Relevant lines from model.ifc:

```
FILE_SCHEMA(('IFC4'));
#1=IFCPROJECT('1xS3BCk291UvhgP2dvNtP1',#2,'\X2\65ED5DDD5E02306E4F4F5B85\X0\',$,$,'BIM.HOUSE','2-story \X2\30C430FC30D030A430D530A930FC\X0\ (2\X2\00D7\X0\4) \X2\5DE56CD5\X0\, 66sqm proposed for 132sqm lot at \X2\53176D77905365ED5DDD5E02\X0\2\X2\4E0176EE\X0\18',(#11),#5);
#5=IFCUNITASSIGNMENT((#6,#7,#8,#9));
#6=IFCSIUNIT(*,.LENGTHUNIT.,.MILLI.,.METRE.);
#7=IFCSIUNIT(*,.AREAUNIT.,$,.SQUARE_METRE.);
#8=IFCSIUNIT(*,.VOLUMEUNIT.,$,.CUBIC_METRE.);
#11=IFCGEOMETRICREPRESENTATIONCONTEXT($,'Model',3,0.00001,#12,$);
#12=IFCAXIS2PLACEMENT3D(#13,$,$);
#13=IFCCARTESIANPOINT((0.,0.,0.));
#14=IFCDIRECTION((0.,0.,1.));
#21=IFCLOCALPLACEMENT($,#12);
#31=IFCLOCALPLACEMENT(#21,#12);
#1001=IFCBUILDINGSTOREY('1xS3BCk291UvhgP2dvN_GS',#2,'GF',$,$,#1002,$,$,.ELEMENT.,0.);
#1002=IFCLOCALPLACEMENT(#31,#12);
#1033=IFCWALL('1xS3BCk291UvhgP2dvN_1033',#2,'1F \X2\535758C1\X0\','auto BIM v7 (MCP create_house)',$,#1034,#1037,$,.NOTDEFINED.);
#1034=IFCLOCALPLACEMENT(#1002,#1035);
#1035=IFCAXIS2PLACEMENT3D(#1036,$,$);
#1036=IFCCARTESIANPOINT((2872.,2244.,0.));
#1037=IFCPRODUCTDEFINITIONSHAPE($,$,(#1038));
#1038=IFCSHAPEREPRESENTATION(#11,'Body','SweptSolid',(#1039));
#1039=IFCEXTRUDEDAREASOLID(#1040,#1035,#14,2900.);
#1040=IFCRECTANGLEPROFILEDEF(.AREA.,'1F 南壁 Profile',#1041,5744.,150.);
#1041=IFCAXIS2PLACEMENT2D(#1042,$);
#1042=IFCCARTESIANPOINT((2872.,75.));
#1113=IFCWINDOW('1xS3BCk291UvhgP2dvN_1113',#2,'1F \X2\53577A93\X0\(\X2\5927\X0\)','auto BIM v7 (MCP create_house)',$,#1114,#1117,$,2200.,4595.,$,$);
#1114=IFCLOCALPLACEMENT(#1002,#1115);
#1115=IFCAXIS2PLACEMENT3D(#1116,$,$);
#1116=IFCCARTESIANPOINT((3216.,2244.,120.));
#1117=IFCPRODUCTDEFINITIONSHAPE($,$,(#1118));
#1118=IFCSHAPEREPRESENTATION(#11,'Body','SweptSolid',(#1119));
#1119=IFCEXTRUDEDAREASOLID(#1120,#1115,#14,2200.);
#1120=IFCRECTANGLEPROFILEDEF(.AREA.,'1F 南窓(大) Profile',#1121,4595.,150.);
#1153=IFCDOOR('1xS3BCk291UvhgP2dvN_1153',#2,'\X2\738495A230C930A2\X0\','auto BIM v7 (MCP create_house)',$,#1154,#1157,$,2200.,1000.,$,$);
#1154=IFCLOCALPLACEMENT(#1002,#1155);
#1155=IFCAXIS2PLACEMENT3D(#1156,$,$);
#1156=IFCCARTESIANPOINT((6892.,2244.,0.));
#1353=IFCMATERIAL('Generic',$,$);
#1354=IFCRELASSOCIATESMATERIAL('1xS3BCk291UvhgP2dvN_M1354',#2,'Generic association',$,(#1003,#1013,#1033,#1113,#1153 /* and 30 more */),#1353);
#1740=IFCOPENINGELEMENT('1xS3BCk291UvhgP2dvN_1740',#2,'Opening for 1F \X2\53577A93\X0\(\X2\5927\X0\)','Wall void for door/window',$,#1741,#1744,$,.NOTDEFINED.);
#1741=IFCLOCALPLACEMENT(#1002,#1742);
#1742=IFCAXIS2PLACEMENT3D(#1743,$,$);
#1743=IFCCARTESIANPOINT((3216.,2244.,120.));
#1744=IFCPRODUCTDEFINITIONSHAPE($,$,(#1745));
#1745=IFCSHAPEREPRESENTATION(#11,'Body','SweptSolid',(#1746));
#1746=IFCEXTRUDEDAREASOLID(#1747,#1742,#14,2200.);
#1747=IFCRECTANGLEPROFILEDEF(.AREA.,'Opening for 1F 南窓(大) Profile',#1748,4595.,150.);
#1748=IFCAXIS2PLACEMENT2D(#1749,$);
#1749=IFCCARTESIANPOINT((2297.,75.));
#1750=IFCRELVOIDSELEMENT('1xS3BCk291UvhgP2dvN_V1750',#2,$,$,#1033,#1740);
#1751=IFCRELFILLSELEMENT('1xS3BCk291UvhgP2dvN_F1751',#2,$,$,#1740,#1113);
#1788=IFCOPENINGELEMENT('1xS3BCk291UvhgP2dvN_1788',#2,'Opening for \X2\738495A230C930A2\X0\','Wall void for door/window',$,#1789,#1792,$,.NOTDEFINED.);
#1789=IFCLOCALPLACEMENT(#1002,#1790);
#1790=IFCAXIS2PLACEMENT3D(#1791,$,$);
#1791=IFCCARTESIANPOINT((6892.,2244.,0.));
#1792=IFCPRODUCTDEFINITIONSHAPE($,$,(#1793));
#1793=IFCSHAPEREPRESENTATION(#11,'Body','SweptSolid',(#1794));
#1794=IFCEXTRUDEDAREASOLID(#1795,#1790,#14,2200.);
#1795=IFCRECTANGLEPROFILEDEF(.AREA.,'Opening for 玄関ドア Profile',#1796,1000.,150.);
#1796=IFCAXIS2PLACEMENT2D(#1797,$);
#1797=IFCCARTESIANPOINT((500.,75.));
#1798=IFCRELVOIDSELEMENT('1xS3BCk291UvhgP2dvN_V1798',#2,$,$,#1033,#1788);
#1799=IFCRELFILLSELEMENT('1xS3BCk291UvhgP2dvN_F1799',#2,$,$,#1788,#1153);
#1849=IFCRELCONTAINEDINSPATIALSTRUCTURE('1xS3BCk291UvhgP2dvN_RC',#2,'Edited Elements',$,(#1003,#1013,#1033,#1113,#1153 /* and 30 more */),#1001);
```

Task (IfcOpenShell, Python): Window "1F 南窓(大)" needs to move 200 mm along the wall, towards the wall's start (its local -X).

```python
import ifcopenshell
import ifcopenshell.api.geometry
import ifcopenshell.util.placement
import ifcopenshell.util.unit

model = ifcopenshell.open("model.ifc")
unit_scale = ifcopenshell.util.unit.calculate_unit_scale(model)

window = model.by_guid("1xS3BCk291UvhgP2dvN_1113")
opening = window.FillsVoids[0].RelatingOpeningElement
wall = opening.VoidsElements[0].RelatingBuildingElement

wall_matrix = ifcopenshell.util.placement.get_local_placement(wall.ObjectPlacement)
shift = wall_matrix[:3, 0] * -0.2 / unit_scale
before = ifcopenshell.util.placement.get_local_placement(window.ObjectPlacement)[:3, 3].copy()

# The window is not placed relative to its opening, so move both.
for product in (opening, window):
    matrix = ifcopenshell.util.placement.get_local_placement(product.ObjectPlacement)
    matrix[:3, 3] += shift
    ifcopenshell.api.geometry.edit_object_placement(model, product=product, matrix=matrix, is_si=False)

after = ifcopenshell.util.placement.get_local_placement(window.ObjectPlacement)[:3, 3]
print("window moved by", (after - before).round(3) + 0.0)

model.write("model_edited.ifc")
```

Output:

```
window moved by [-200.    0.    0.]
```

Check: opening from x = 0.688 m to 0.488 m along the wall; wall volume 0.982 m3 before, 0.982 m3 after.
